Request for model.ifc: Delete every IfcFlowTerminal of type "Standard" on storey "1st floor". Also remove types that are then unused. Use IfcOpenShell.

First a look at what the model holds.

```python
import ifcopenshell
import ifcopenshell.util.element

model = ifcopenshell.open("model.ifc")
print(model.schema)
storey = next(s for s in model.by_type("IfcBuildingStorey") if s.Name == "1st floor")
terminals = [e for e in ifcopenshell.util.element.get_decomposition(storey) if e.is_a("IfcFlowTerminal")]
seen = {}
for e in terminals:
    element_type = ifcopenshell.util.element.get_type(e)
    name = element_type.Name if element_type not in (None, e) else None
    seen[name] = seen.get(name, 0) + 1
for name, count in sorted(seen.items(), key=str):
    print(count, "x", name)
```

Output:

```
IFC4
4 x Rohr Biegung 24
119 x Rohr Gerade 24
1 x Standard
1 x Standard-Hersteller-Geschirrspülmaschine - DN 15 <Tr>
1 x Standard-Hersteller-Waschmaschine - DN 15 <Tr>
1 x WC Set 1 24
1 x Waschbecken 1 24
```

```python
import ifcopenshell
import ifcopenshell.api.root
import ifcopenshell.util.element

model = ifcopenshell.open("model.ifc")

storey = next(s for s in model.by_type("IfcBuildingStorey") if s.Name == "1st floor")
terminals = [e for e in ifcopenshell.util.element.get_decomposition(storey) if e.is_a("IfcFlowTerminal")]
targets = [e for e in terminals if (t := ifcopenshell.util.element.get_type(e)) not in (None, e) and t.Name == "Standard"]
types = {ifcopenshell.util.element.get_type(e) for e in targets} - {None, *targets}

for e in targets:
    ifcopenshell.api.root.remove_product(model, product=e)
print(len(targets), "removed")

unused = [t for t in types if not ifcopenshell.util.element.get_types(t)]
for t in unused:
    ifcopenshell.api.root.remove_product(model, product=t)
print(len(unused), "unused types removed")

model.write("model_v2.ifc")
```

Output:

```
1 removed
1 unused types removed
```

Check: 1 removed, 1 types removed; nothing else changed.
